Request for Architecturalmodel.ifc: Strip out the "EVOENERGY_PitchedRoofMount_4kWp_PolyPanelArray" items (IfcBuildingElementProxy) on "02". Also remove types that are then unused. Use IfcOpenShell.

First a look at what the model holds.

```python
import ifcopenshell
import ifcopenshell.util.element

model = ifcopenshell.open("Architecturalmodel.ifc")
print(model.schema)
storey = next(s for s in model.by_type("IfcBuildingStorey") if s.Name == "02")
proxies = [e for e in ifcopenshell.util.element.get_decomposition(storey) if e.is_a("IfcBuildingElementProxy")]
seen = {}
for e in proxies:
    element_type = ifcopenshell.util.element.get_type(e)
    name = element_type.Name if element_type not in (None, e) else None
    seen[name] = seen.get(name, 0) + 1
for name, count in sorted(seen.items(), key=str):
    print(count, "x", name)
```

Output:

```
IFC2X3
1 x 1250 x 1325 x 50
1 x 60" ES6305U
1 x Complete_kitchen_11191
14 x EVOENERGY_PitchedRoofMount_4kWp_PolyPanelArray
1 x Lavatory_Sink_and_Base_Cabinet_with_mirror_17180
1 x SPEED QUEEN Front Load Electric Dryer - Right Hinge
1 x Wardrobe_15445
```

```python
import ifcopenshell
import ifcopenshell.api.root
import ifcopenshell.util.element

model = ifcopenshell.open("Architecturalmodel.ifc")

storey = next(s for s in model.by_type("IfcBuildingStorey") if s.Name == "02")
proxies = [e for e in ifcopenshell.util.element.get_decomposition(storey) if e.is_a("IfcBuildingElementProxy")]
targets = [e for e in proxies if (t := ifcopenshell.util.element.get_type(e)) not in (None, e) and t.Name == "EVOENERGY_PitchedRoofMount_4kWp_PolyPanelArray"]
types = {ifcopenshell.util.element.get_type(e) for e in targets} - {None, *targets}

for e in targets:
    ifcopenshell.api.root.remove_product(model, product=e)
print(len(targets), "removed")

unused = [t for t in types if not ifcopenshell.util.element.get_types(t)]
for t in unused:
    ifcopenshell.api.root.remove_product(model, product=t)
print(len(unused), "unused types removed")

model.write("Architecturalmodel_rev.ifc")
```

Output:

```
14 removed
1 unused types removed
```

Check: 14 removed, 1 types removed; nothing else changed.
